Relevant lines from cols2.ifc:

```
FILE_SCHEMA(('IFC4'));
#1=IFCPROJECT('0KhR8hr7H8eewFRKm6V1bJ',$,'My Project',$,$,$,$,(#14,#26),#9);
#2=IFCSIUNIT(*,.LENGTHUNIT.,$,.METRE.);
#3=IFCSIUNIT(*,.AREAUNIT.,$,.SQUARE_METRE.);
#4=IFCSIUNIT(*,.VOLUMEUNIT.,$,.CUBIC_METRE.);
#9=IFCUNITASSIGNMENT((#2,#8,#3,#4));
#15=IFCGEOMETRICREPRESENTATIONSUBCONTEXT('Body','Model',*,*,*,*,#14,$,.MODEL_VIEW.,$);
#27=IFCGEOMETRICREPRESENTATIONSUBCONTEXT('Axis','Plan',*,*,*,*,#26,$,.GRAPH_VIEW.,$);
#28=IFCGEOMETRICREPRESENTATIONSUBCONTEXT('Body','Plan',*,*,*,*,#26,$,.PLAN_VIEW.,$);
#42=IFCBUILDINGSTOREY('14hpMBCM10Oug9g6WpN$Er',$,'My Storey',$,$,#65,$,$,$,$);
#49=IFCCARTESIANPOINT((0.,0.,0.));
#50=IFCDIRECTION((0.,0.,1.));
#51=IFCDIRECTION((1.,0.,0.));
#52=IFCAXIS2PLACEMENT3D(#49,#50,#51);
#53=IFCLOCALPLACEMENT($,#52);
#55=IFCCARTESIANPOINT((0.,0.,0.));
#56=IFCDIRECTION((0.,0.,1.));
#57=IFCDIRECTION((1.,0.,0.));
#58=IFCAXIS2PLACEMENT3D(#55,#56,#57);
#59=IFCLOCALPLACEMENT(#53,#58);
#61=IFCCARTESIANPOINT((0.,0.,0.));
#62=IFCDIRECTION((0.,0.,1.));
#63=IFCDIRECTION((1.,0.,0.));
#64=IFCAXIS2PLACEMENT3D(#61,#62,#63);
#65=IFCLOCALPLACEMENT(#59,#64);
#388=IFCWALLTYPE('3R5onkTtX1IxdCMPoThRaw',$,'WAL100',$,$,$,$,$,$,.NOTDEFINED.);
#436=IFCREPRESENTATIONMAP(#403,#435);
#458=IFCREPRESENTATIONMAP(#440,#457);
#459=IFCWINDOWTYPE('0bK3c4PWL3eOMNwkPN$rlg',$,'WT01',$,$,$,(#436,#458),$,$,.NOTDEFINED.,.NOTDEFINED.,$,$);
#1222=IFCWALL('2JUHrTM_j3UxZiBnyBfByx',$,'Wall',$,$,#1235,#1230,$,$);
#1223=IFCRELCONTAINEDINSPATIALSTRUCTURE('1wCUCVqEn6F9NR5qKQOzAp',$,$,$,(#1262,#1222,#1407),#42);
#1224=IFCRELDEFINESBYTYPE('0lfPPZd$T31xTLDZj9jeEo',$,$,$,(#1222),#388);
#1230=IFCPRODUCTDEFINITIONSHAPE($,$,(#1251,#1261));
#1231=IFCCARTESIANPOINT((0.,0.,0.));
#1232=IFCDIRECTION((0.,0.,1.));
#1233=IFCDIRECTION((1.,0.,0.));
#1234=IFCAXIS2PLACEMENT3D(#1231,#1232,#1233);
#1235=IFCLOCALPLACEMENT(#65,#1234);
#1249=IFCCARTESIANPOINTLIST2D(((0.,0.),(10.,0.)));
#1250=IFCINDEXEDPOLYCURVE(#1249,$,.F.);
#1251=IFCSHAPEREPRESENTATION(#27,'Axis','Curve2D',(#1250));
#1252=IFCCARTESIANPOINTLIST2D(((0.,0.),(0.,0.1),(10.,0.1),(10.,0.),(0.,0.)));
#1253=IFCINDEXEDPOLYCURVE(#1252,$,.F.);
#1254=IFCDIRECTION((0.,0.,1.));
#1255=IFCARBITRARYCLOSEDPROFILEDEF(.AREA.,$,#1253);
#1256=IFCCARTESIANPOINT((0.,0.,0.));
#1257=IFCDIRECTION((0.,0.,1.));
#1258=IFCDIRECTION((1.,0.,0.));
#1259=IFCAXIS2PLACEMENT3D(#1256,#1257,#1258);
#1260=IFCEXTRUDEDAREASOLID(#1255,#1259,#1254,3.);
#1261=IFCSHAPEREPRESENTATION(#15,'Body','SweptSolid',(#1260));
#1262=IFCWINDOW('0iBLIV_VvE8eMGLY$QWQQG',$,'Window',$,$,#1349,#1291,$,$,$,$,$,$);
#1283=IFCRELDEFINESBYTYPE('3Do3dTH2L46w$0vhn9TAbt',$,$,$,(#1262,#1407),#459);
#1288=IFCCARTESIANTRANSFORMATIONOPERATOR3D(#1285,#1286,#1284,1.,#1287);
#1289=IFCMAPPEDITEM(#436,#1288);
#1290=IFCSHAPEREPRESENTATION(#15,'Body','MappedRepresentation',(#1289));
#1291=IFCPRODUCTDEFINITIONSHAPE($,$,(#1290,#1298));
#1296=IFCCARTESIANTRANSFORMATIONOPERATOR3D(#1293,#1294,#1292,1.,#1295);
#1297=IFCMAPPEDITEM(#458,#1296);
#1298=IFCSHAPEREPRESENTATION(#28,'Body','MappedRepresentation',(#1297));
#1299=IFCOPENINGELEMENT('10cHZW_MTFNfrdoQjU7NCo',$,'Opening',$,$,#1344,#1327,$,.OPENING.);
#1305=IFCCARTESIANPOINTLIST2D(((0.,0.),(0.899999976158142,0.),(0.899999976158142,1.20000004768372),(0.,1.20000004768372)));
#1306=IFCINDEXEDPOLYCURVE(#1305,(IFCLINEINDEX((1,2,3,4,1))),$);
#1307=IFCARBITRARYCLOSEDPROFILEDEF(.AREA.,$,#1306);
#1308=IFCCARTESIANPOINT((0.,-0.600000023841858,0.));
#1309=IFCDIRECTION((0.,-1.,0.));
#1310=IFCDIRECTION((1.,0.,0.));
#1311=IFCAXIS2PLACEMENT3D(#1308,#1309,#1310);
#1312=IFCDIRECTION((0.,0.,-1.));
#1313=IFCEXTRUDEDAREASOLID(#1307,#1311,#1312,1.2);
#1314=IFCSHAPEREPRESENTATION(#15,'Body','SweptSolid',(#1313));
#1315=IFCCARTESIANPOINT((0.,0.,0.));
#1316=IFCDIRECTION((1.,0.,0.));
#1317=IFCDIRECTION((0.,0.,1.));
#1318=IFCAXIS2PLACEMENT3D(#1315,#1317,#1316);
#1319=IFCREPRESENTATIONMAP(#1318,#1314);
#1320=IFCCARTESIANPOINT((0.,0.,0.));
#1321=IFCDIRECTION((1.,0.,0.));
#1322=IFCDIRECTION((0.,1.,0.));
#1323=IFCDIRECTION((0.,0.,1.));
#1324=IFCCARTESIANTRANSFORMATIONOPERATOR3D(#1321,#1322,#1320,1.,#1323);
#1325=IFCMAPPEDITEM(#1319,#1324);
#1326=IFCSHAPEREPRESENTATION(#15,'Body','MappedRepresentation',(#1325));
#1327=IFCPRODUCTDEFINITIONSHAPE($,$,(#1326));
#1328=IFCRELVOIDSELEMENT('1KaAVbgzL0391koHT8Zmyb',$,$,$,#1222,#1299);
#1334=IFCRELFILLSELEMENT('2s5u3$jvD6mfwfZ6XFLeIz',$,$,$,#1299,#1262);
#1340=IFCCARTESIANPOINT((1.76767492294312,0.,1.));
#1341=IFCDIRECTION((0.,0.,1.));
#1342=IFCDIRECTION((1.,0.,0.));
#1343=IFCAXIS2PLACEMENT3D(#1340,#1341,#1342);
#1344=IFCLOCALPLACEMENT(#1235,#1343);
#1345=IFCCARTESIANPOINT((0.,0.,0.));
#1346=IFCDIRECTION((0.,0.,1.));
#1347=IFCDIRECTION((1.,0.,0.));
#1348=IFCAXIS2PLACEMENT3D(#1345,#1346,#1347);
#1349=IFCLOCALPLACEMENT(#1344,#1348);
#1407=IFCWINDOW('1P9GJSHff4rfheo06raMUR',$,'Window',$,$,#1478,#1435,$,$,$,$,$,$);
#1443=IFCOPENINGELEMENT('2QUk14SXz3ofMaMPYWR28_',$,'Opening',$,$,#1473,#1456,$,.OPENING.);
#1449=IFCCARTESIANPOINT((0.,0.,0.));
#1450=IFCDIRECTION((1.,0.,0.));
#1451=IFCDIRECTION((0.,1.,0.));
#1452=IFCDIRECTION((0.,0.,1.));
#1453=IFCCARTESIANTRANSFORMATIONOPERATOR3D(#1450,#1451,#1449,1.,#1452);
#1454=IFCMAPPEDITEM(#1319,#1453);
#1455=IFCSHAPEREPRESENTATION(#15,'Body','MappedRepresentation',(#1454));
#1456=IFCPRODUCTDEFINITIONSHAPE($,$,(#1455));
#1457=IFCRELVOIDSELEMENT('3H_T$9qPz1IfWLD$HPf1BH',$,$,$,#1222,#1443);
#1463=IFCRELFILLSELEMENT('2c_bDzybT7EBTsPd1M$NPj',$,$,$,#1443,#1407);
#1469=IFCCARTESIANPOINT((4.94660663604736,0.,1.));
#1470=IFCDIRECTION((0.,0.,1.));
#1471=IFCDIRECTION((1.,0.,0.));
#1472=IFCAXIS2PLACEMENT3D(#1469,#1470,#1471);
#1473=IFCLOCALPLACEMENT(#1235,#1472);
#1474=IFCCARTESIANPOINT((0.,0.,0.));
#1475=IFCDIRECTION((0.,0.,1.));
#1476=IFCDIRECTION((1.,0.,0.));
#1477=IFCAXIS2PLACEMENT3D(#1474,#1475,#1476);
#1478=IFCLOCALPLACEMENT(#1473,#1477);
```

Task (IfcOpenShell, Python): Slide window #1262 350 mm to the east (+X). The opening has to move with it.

```python
import ifcopenshell
import ifcopenshell.api.geometry
import ifcopenshell.util.placement
import ifcopenshell.util.unit

model = ifcopenshell.open("cols2.ifc")
unit_scale = ifcopenshell.util.unit.calculate_unit_scale(model)

window = model.by_id(1262)
opening = window.FillsVoids[0].RelatingOpeningElement
wall = opening.VoidsElements[0].RelatingBuildingElement

wall_matrix = ifcopenshell.util.placement.get_local_placement(wall.ObjectPlacement)
shift = wall_matrix[:3, 0] * 0.35 / unit_scale
before = ifcopenshell.util.placement.get_local_placement(window.ObjectPlacement)[:3, 3].copy()

# The window is placed relative to its opening, so it follows when the opening moves.
matrix = ifcopenshell.util.placement.get_local_placement(opening.ObjectPlacement)
matrix[:3, 3] += shift
ifcopenshell.api.geometry.edit_object_placement(
    model, product=opening, matrix=matrix, is_si=False, should_transform_children=True
)

after = ifcopenshell.util.placement.get_local_placement(window.ObjectPlacement)[:3, 3]
print("window moved by", (after - before).round(3) + 0.0)

model.write("cols2-out.ifc")
```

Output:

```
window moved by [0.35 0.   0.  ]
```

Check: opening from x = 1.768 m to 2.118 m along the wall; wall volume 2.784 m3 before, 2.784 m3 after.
